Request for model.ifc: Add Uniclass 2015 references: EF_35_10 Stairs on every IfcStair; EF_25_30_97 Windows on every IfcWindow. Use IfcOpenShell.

First a look at what the model holds.

```python
import ifcopenshell

model = ifcopenshell.open("model.ifc")
print(model.schema)
print("classifications:", [c.Name for c in model.by_type("IfcClassification")])
for ifc_class in ("IfcDoor", "IfcRoof", "IfcStair", "IfcWall", "IfcWindow"):
    print(ifc_class, len(model.by_type(ifc_class)))
```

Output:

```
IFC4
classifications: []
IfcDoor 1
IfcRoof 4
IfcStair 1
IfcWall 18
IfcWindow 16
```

```python
import ifcopenshell
import ifcopenshell.api.classification

model = ifcopenshell.open("model.ifc")

system = ifcopenshell.api.classification.add_classification(model, classification="Uniclass 2015")

codes = {
    "IfcStair": ("EF_35_10", "Stairs"),
    "IfcWindow": ("EF_25_30_97", "Windows"),
}
for ifc_class, (code, name) in codes.items():
    products = model.by_type(ifc_class)
    ifcopenshell.api.classification.add_reference(
        model, products=products, classification=system, identification=code, name=name
    )
    print(code, len(products))

model.write("model_updated.ifc")
```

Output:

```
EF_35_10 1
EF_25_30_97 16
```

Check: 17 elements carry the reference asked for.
